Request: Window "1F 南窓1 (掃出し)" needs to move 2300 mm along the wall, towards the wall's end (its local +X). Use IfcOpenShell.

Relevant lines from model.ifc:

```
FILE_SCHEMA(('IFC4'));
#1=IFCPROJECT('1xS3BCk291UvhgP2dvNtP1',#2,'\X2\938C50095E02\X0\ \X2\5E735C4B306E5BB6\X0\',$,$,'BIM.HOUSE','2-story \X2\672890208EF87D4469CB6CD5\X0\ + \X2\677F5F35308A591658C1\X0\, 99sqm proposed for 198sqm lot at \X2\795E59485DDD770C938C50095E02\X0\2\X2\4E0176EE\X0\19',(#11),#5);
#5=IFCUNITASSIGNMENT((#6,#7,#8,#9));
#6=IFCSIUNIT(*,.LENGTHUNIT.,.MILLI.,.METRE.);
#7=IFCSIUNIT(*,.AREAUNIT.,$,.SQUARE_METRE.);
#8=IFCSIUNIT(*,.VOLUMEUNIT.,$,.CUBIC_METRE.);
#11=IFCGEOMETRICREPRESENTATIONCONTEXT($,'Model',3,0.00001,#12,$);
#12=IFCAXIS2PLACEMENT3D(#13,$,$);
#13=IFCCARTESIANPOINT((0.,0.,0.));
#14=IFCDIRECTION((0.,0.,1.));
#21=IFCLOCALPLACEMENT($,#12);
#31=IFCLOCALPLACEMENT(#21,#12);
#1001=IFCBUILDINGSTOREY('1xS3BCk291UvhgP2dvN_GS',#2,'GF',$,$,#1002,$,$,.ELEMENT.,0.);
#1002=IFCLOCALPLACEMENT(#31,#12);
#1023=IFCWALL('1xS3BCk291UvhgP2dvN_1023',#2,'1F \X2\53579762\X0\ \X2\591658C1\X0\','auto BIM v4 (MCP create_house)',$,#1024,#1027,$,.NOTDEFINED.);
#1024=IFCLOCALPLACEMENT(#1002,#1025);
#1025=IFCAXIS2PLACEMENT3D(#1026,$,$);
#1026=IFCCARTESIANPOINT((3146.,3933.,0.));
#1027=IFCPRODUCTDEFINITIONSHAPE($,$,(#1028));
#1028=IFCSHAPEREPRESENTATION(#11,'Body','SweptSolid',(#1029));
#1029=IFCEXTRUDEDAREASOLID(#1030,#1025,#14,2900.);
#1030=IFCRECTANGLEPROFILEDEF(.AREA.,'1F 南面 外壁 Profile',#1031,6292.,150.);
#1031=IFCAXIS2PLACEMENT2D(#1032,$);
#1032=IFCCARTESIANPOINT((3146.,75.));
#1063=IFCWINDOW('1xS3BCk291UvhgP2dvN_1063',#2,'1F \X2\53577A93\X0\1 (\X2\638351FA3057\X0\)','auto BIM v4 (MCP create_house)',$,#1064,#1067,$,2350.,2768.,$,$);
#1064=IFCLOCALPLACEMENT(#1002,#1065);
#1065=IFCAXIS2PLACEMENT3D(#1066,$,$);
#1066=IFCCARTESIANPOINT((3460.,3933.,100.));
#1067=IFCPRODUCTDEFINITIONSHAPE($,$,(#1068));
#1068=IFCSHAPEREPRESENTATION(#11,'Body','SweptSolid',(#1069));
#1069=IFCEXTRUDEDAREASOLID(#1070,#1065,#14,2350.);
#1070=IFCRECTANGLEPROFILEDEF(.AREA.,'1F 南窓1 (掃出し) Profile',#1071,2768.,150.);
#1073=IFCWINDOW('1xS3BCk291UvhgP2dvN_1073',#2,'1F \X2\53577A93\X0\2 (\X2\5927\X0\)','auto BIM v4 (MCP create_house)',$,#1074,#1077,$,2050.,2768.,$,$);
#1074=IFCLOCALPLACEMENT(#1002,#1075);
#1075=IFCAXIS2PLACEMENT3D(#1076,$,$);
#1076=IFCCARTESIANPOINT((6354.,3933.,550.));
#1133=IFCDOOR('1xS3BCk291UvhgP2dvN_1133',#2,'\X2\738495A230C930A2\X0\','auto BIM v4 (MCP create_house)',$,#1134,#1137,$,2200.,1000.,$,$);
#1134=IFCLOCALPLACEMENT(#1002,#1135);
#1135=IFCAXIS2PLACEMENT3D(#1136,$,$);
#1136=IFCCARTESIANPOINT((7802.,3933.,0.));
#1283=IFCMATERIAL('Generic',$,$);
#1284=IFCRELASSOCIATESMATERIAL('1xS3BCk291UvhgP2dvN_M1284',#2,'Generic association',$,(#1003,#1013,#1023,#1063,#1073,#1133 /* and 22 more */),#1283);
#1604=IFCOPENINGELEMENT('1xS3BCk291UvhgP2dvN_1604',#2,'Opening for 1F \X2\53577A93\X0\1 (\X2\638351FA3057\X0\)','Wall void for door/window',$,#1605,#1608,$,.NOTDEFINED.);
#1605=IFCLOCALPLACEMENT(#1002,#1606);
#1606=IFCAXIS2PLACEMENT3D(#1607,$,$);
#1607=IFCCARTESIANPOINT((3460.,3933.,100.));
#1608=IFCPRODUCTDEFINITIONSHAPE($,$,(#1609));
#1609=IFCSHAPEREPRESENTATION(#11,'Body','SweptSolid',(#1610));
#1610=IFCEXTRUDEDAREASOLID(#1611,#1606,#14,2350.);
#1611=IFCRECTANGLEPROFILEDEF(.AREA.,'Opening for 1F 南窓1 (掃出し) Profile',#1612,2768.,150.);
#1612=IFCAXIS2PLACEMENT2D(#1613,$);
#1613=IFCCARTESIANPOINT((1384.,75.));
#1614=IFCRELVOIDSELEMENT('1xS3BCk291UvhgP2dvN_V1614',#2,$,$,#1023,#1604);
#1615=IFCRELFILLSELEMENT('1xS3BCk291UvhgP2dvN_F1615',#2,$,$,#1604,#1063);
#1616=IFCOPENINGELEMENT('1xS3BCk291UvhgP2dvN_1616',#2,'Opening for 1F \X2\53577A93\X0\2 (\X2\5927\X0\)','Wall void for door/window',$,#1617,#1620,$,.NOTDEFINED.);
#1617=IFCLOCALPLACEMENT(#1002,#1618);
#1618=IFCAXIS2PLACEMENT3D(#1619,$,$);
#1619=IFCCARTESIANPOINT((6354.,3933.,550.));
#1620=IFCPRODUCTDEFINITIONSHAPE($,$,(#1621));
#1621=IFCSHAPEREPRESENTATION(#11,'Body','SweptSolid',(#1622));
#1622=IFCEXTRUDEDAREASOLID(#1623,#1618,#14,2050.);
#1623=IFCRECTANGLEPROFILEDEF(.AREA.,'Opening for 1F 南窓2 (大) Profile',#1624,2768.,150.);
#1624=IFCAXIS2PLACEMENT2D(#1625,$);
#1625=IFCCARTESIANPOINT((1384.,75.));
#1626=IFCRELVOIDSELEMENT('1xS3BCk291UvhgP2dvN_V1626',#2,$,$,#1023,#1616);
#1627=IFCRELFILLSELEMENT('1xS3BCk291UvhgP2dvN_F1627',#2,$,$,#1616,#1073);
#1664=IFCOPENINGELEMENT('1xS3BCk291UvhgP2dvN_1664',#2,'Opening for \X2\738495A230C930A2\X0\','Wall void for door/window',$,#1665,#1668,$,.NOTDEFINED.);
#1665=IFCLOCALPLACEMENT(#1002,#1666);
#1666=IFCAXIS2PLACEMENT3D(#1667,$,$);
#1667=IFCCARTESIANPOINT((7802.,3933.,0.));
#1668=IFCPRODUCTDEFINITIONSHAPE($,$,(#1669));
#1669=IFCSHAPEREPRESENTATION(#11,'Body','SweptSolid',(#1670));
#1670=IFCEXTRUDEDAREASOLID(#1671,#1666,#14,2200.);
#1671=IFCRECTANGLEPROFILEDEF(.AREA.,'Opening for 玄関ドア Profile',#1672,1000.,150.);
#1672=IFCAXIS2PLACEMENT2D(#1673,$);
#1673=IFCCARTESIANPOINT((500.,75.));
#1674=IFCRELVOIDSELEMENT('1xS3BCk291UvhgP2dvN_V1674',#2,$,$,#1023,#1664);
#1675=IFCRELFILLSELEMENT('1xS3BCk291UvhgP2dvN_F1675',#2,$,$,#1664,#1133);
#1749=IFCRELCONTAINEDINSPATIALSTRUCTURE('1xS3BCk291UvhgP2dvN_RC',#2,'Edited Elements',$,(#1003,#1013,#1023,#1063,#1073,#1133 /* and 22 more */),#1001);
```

```python
import ifcopenshell
import ifcopenshell.api.geometry
import ifcopenshell.util.placement

model = ifcopenshell.open("model.ifc")

window = model.by_guid("1xS3BCk291UvhgP2dvN_1063")
opening = window.FillsVoids[0].RelatingOpeningElement
wall = opening.VoidsElements[0].RelatingBuildingElement

wall_matrix = ifcopenshell.util.placement.get_local_placement(wall.ObjectPlacement)
shift = wall_matrix[:3, 0] * 2300.0
before = ifcopenshell.util.placement.get_local_placement(window.ObjectPlacement)[:3, 3].copy()

# The window is not placed relative to its opening, so move both.
for product in (opening, window):
    matrix = ifcopenshell.util.placement.get_local_placement(product.ObjectPlacement)
    matrix[:3, 3] += shift
    ifcopenshell.api.geometry.edit_object_placement(model, product=product, matrix=matrix, is_si=False)

after = ifcopenshell.util.placement.get_local_placement(window.ObjectPlacement)[:3, 3]
print("window moved by", (after - before).round(3) + 0.0)

model.write("model-out.ifc")
```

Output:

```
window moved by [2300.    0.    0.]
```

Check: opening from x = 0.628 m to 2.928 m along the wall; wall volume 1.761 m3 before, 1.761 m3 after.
